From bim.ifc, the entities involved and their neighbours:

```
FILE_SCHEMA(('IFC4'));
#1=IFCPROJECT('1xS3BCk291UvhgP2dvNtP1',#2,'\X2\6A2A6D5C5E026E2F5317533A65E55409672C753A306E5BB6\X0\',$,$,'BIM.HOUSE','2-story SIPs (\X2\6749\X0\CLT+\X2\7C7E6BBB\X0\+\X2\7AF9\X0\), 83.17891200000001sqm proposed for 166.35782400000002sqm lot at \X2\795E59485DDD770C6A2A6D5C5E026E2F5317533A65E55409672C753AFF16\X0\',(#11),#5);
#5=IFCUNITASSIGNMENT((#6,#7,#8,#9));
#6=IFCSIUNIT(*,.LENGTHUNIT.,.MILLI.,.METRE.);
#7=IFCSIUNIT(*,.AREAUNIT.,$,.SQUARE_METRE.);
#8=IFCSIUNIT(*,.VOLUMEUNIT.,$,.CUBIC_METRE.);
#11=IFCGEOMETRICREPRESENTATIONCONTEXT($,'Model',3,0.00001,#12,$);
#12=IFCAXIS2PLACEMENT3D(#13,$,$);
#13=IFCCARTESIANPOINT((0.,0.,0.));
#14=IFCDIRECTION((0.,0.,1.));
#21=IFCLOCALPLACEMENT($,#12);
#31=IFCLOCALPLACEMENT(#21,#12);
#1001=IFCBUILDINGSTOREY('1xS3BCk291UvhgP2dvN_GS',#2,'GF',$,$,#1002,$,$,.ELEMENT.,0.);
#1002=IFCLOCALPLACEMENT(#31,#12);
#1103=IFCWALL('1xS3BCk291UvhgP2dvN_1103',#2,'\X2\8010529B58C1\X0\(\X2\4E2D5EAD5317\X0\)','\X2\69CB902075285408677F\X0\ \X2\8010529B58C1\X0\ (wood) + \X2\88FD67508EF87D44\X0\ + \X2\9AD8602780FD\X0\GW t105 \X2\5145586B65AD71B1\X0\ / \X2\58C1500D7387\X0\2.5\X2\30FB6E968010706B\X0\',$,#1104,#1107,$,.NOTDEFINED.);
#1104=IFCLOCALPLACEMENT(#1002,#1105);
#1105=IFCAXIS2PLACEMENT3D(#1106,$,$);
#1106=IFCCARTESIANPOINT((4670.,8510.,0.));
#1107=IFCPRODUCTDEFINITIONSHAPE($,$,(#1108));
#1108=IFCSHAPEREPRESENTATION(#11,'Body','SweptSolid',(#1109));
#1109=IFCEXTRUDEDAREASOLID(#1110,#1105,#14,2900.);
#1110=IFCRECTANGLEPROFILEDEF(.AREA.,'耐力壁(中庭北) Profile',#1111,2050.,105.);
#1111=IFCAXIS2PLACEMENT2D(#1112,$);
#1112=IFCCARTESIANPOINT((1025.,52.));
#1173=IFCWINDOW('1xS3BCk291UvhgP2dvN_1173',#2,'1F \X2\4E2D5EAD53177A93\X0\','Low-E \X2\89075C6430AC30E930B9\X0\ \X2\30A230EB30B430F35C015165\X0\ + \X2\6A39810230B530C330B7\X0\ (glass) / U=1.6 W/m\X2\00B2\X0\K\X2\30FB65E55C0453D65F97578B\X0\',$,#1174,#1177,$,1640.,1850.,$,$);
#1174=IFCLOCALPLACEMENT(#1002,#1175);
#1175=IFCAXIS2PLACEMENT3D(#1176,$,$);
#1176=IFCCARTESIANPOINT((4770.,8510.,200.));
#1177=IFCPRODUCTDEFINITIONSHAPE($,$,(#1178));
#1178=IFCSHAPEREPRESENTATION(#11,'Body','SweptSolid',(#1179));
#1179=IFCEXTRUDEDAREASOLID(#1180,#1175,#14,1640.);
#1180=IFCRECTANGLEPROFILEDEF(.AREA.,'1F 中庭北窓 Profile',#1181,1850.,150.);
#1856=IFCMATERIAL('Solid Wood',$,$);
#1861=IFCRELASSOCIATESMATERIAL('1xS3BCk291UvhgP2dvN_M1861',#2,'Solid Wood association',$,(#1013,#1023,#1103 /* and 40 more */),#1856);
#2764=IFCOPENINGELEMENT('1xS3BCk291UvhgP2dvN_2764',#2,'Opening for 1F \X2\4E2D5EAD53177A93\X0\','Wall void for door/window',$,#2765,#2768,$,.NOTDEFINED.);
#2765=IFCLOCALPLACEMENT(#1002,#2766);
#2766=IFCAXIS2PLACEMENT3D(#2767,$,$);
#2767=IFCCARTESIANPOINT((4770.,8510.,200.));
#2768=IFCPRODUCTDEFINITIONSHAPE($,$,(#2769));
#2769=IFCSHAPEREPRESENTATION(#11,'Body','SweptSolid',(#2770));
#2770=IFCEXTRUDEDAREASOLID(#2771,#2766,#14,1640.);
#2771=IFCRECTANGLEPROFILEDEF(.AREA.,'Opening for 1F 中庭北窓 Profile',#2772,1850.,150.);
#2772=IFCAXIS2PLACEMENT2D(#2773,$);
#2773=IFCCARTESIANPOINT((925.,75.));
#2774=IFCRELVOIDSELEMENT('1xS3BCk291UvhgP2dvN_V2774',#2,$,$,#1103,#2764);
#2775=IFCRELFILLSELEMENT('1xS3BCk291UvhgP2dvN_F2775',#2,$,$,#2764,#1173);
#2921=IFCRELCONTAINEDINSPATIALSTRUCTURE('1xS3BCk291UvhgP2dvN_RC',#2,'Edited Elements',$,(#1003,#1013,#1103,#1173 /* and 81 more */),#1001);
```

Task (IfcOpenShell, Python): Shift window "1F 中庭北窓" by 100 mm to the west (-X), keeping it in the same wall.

```python
import ifcopenshell
import ifcopenshell.api.geometry
import ifcopenshell.util.placement
import ifcopenshell.util.unit

model = ifcopenshell.open("bim.ifc")
unit_scale = ifcopenshell.util.unit.calculate_unit_scale(model)

window = model.by_guid("1xS3BCk291UvhgP2dvN_1173")
opening = window.FillsVoids[0].RelatingOpeningElement
wall = opening.VoidsElements[0].RelatingBuildingElement

wall_matrix = ifcopenshell.util.placement.get_local_placement(wall.ObjectPlacement)
shift = wall_matrix[:3, 0] * -0.1 / unit_scale
before = ifcopenshell.util.placement.get_local_placement(window.ObjectPlacement)[:3, 3].copy()

# The window is not placed relative to its opening, so move both.
for product in (opening, window):
    matrix = ifcopenshell.util.placement.get_local_placement(product.ObjectPlacement)
    matrix[:3, 3] += shift
    ifcopenshell.api.geometry.edit_object_placement(model, product=product, matrix=matrix, is_si=False)

after = ifcopenshell.util.placement.get_local_placement(window.ObjectPlacement)[:3, 3]
print("window moved by", (after - before).round(3) + 0.0)

model.write("bim_rev.ifc")
```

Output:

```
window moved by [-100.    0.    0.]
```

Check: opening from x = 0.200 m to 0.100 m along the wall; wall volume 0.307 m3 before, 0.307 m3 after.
